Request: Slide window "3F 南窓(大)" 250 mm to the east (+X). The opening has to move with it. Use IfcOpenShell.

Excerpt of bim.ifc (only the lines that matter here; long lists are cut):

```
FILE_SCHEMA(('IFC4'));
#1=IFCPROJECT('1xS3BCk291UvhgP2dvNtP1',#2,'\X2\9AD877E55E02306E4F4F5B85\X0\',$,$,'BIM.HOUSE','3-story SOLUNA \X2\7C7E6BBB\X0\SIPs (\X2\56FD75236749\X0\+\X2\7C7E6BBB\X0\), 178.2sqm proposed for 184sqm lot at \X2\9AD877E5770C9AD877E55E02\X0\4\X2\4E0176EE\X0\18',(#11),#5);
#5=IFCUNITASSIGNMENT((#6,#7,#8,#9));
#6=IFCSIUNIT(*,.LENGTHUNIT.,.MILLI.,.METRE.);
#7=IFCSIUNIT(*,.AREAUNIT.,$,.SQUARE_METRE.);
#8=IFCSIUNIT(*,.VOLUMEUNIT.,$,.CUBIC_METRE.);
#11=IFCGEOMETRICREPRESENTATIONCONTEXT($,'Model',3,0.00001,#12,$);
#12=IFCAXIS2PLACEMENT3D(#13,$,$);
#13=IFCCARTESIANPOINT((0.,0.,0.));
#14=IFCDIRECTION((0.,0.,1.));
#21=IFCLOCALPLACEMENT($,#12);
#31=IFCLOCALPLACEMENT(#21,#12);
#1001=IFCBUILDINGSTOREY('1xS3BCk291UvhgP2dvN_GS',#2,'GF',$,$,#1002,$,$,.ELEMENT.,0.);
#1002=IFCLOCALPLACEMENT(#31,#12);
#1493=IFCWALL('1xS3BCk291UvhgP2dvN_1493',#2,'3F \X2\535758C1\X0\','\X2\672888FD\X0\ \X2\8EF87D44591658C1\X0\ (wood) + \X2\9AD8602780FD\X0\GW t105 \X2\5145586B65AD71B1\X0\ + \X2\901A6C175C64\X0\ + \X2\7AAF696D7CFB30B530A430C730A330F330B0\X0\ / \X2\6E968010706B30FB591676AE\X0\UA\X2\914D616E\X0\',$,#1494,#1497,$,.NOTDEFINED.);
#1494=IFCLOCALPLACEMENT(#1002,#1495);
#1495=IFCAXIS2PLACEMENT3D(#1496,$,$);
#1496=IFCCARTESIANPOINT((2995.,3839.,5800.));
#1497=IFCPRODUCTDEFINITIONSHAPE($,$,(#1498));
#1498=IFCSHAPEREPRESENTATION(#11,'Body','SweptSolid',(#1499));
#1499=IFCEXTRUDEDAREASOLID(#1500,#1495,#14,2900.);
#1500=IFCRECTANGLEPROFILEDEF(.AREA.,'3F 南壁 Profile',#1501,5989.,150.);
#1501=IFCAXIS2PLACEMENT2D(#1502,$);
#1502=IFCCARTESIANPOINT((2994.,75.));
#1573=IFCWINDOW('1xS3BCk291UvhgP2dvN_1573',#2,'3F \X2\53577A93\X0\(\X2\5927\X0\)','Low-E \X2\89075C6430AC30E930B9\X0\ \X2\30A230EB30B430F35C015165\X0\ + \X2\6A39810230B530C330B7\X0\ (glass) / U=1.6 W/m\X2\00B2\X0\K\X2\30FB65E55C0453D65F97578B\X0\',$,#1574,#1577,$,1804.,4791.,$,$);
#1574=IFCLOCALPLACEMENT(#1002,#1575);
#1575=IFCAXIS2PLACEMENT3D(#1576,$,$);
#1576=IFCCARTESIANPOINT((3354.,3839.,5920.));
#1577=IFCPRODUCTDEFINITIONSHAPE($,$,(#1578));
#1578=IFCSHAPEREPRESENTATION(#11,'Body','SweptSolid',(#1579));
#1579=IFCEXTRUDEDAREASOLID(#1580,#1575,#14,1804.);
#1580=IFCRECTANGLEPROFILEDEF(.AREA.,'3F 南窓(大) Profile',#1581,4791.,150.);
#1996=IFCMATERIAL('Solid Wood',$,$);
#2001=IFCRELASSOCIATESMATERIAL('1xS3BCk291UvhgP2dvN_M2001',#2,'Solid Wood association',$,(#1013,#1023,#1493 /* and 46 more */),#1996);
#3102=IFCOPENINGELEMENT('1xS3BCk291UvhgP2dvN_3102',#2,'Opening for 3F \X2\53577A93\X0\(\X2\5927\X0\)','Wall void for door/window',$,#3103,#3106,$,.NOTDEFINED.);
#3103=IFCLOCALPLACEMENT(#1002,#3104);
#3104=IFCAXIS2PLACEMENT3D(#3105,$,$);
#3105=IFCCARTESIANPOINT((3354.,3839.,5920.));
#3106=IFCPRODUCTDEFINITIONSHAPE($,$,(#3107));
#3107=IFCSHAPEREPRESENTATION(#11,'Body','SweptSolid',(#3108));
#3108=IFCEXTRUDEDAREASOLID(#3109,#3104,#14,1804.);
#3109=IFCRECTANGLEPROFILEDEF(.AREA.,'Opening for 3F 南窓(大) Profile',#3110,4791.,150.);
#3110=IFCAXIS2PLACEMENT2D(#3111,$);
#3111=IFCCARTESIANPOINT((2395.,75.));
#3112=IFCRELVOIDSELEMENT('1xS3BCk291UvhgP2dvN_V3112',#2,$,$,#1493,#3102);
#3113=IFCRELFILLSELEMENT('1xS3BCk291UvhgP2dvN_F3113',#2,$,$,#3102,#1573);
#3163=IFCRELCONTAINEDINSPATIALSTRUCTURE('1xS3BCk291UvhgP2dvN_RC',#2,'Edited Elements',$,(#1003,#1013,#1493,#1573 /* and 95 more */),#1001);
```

```python
import ifcopenshell
import ifcopenshell.api.geometry
import ifcopenshell.util.placement

model = ifcopenshell.open("bim.ifc")

window = model.by_guid("1xS3BCk291UvhgP2dvN_1573")
opening = window.FillsVoids[0].RelatingOpeningElement
wall = opening.VoidsElements[0].RelatingBuildingElement

wall_matrix = ifcopenshell.util.placement.get_local_placement(wall.ObjectPlacement)
shift = wall_matrix[:3, 0] * 250.0
before = ifcopenshell.util.placement.get_local_placement(window.ObjectPlacement)[:3, 3].copy()

# The window is not placed relative to its opening, so move both.
for product in (opening, window):
    matrix = ifcopenshell.util.placement.get_local_placement(product.ObjectPlacement)
    matrix[:3, 3] += shift
    ifcopenshell.api.geometry.edit_object_placement(model, product=product, matrix=matrix, is_si=False)

after = ifcopenshell.util.placement.get_local_placement(window.ObjectPlacement)[:3, 3]
print("window moved by", (after - before).round(3) + 0.0)

model.write("bim_updated.ifc")
```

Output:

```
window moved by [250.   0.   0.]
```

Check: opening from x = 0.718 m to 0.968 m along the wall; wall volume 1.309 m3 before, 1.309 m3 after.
